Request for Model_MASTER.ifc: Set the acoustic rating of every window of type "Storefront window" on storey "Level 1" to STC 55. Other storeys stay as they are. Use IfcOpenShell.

First a look at what the model holds.

```python
import ifcopenshell
import ifcopenshell.util.element

model = ifcopenshell.open("Model_MASTER.ifc")
print(model.schema)
storey = next(s for s in model.by_type("IfcBuildingStorey") if s.Name == "Level 1")
windows = [e for e in ifcopenshell.util.element.get_decomposition(storey) if e.is_a("IfcWindow")]
seen = {}
for e in windows:
    element_type = ifcopenshell.util.element.get_type(e)
    key = (element_type.Name if element_type != e and element_type else None, ifcopenshell.util.element.get_pset(e, "Pset_WindowCommon", "AcousticRating"))
    seen[key] = seen.get(key, 0) + 1
for (name, value), count in sorted(seen.items(), key=str):
    print(count, "x", name, "|", value)
```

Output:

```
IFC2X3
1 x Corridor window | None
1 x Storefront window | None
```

```python
import ifcopenshell
import ifcopenshell.api.pset
import ifcopenshell.util.element

model = ifcopenshell.open("Model_MASTER.ifc")

storey = next(s for s in model.by_type("IfcBuildingStorey") if s.Name == "Level 1")
windows = [e for e in ifcopenshell.util.element.get_decomposition(storey) if e.is_a("IfcWindow")]

count = 0
for e in windows:
    element_type = ifcopenshell.util.element.get_type(e)
    if element_type in (None, e) or element_type.Name != "Storefront window":
        continue
    # add_pset returns the element's existing set when there is one.
    pset = ifcopenshell.api.pset.add_pset(model, product=e, name="Pset_WindowCommon")
    ifcopenshell.api.pset.edit_pset(model, pset=pset, properties={"AcousticRating": "STC 55"})
    count += 1

print(count, "windows updated")

model.write("Model_MASTER_edited.ifc")
```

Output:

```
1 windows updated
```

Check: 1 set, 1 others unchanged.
